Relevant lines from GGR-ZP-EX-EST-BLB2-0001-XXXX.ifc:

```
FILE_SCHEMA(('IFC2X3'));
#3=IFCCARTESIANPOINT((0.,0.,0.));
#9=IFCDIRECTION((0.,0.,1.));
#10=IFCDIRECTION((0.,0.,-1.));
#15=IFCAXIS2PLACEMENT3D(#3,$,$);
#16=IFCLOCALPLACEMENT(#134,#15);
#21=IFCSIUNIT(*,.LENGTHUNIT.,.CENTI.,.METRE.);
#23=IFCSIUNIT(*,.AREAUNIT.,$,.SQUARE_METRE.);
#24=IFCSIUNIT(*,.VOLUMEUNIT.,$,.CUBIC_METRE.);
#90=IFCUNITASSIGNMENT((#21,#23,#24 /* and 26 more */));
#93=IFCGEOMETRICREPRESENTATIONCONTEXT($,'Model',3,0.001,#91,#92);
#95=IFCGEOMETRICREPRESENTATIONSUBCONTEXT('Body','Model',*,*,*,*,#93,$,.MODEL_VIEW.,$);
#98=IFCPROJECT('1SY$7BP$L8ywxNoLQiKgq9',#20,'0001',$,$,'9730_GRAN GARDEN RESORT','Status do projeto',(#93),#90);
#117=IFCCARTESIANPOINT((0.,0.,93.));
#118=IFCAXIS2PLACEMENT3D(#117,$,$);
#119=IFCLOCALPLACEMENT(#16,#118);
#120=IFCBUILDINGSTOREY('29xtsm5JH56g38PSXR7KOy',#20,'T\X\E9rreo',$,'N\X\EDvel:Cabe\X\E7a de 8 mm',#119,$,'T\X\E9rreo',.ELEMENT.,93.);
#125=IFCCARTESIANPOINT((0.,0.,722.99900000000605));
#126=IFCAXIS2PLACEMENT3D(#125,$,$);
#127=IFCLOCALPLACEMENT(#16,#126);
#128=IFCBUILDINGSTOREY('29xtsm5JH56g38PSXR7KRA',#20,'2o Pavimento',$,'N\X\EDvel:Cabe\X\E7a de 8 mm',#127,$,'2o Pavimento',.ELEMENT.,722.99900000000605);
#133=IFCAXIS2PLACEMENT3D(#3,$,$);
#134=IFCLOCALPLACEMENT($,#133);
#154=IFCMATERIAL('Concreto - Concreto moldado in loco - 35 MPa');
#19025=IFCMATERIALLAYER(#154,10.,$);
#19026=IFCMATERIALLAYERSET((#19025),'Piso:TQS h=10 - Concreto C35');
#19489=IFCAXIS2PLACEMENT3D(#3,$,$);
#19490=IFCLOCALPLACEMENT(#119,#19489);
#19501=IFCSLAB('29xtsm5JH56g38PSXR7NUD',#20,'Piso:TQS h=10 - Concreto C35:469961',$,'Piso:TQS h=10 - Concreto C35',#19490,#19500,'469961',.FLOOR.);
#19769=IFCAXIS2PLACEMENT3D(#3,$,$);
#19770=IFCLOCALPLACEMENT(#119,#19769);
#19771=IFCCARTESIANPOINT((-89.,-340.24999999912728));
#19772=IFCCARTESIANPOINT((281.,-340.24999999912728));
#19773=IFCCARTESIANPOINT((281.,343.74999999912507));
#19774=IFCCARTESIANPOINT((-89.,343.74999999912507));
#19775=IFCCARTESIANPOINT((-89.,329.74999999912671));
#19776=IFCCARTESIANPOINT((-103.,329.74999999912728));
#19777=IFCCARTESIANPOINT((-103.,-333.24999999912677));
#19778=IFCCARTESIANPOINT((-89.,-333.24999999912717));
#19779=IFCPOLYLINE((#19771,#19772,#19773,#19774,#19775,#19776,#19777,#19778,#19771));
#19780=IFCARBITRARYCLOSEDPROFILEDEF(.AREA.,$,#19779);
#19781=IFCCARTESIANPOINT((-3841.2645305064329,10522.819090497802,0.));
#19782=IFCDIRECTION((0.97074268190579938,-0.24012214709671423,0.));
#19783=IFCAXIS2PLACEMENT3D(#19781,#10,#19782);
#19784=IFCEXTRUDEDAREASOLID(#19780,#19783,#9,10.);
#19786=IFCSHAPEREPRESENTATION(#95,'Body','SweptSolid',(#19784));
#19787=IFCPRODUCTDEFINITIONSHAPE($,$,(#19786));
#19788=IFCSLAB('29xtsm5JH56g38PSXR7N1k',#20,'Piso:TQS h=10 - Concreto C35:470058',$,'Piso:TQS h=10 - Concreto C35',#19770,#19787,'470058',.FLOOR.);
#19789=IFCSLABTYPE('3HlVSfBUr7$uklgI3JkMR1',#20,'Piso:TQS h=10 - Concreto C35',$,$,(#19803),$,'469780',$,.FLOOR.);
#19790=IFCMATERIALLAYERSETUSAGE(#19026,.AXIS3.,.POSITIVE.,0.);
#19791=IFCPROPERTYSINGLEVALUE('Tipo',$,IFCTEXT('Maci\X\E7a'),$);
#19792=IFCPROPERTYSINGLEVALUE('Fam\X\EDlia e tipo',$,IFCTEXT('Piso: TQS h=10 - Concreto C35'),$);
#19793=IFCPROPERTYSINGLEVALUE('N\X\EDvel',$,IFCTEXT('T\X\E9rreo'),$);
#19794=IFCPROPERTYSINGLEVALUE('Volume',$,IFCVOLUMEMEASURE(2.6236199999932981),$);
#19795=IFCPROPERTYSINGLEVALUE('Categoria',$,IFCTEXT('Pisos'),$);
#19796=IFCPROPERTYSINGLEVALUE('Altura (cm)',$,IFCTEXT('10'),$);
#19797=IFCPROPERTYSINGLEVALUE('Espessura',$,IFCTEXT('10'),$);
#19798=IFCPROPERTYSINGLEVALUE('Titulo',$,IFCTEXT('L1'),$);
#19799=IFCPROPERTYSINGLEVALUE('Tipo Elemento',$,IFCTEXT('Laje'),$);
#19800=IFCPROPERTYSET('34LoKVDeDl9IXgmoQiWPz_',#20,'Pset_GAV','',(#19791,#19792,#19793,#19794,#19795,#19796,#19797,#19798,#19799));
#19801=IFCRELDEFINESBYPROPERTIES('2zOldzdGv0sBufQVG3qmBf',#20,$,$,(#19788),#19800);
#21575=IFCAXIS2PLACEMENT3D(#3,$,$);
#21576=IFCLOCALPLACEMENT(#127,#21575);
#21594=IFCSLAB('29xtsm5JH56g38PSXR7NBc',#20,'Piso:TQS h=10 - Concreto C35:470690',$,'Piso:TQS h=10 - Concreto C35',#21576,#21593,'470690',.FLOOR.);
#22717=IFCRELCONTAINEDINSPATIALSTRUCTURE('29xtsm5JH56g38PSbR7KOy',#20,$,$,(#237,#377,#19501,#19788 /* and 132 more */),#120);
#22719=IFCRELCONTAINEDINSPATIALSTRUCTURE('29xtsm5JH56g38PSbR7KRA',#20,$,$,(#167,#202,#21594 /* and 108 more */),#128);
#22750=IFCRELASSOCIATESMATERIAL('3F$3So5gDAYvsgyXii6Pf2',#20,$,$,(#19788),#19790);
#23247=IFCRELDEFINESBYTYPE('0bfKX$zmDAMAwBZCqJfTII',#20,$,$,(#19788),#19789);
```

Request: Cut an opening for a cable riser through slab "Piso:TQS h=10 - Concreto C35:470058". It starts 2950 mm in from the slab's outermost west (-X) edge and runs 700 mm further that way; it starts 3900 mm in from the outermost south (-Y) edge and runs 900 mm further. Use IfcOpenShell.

```python
import numpy as np
import ifcopenshell
import ifcopenshell.api.feature
import ifcopenshell.api.geometry
import ifcopenshell.api.pset
import ifcopenshell.api.root
import ifcopenshell.geom
import ifcopenshell.util.element
import ifcopenshell.util.placement
import ifcopenshell.util.representation
import ifcopenshell.util.shape
import ifcopenshell.util.unit

model = ifcopenshell.open("GGR-ZP-EX-EST-BLB2-0001-XXXX.ifc")
unit_scale = ifcopenshell.util.unit.calculate_unit_scale(model)
volume_scale = ifcopenshell.util.unit.calculate_unit_scale(model, "VOLUMEUNIT")
settings = ifcopenshell.geom.settings()


def volume(element):
    """Net volume in cubic metres, openings subtracted."""
    shape = ifcopenshell.geom.create_shape(settings, element)
    return ifcopenshell.util.shape.get_volume(shape.geometry)


slab = model.by_guid("29xtsm5JH56g38PSXR7N1k")
before = volume(slab)

# Extent in the slab's own axes, in metres. The edges named are its -X and -Y sides.
slab_shape = ifcopenshell.geom.create_shape(settings, slab)
vertices = ifcopenshell.util.shape.get_vertices(slab_shape.geometry)
x_min, y_min, bottom = vertices.min(axis=0)
top = vertices[:, 2].max()

opening = ifcopenshell.api.root.create_entity(model, ifc_class="IfcOpeningElement", name="Cable riser opening")
context = ifcopenshell.util.representation.get_context(model, "Model", "Body", "MODEL_VIEW")
width, depth = 0.7, 0.9
outline = [(0.0, 0.0), (width, 0.0), (width, depth), (0.0, depth), (0.0, 0.0)]
# Overshoot both faces by 50 mm so the cut is clean.
shape = ifcopenshell.api.geometry.add_slab_representation(
    model, context=context, depth=top - bottom + 0.1, polyline=outline
)
ifcopenshell.api.geometry.assign_representation(model, product=opening, representation=shape)

matrix = ifcopenshell.util.placement.get_local_placement(slab.ObjectPlacement)
matrix[:, 3] = matrix @ np.append(np.array([x_min + 2.95, y_min + 3.9, bottom - 0.05]) / unit_scale, 1.0)
ifcopenshell.api.geometry.edit_object_placement(model, product=opening, matrix=matrix, is_si=False)
ifcopenshell.api.feature.add_feature(model, feature=opening, element=slab)

after = volume(slab)

# Update the slab's stored quantities.
pset = model.by_id(ifcopenshell.util.element.get_pset(slab, "Pset_GAV", should_inherit=False)["id"])
ifcopenshell.api.pset.edit_pset(model, pset=pset, properties={
    "Volume": model.create_entity("IfcVolumeMeasure", after / volume_scale),
})

print(f"slab volume {before:.3f} -> {after:.3f} m3")

model.write("GGR-ZP-EX-EST-BLB2-0001-XXXX-out.ifc")
```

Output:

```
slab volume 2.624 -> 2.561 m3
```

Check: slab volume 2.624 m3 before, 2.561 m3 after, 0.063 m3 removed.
